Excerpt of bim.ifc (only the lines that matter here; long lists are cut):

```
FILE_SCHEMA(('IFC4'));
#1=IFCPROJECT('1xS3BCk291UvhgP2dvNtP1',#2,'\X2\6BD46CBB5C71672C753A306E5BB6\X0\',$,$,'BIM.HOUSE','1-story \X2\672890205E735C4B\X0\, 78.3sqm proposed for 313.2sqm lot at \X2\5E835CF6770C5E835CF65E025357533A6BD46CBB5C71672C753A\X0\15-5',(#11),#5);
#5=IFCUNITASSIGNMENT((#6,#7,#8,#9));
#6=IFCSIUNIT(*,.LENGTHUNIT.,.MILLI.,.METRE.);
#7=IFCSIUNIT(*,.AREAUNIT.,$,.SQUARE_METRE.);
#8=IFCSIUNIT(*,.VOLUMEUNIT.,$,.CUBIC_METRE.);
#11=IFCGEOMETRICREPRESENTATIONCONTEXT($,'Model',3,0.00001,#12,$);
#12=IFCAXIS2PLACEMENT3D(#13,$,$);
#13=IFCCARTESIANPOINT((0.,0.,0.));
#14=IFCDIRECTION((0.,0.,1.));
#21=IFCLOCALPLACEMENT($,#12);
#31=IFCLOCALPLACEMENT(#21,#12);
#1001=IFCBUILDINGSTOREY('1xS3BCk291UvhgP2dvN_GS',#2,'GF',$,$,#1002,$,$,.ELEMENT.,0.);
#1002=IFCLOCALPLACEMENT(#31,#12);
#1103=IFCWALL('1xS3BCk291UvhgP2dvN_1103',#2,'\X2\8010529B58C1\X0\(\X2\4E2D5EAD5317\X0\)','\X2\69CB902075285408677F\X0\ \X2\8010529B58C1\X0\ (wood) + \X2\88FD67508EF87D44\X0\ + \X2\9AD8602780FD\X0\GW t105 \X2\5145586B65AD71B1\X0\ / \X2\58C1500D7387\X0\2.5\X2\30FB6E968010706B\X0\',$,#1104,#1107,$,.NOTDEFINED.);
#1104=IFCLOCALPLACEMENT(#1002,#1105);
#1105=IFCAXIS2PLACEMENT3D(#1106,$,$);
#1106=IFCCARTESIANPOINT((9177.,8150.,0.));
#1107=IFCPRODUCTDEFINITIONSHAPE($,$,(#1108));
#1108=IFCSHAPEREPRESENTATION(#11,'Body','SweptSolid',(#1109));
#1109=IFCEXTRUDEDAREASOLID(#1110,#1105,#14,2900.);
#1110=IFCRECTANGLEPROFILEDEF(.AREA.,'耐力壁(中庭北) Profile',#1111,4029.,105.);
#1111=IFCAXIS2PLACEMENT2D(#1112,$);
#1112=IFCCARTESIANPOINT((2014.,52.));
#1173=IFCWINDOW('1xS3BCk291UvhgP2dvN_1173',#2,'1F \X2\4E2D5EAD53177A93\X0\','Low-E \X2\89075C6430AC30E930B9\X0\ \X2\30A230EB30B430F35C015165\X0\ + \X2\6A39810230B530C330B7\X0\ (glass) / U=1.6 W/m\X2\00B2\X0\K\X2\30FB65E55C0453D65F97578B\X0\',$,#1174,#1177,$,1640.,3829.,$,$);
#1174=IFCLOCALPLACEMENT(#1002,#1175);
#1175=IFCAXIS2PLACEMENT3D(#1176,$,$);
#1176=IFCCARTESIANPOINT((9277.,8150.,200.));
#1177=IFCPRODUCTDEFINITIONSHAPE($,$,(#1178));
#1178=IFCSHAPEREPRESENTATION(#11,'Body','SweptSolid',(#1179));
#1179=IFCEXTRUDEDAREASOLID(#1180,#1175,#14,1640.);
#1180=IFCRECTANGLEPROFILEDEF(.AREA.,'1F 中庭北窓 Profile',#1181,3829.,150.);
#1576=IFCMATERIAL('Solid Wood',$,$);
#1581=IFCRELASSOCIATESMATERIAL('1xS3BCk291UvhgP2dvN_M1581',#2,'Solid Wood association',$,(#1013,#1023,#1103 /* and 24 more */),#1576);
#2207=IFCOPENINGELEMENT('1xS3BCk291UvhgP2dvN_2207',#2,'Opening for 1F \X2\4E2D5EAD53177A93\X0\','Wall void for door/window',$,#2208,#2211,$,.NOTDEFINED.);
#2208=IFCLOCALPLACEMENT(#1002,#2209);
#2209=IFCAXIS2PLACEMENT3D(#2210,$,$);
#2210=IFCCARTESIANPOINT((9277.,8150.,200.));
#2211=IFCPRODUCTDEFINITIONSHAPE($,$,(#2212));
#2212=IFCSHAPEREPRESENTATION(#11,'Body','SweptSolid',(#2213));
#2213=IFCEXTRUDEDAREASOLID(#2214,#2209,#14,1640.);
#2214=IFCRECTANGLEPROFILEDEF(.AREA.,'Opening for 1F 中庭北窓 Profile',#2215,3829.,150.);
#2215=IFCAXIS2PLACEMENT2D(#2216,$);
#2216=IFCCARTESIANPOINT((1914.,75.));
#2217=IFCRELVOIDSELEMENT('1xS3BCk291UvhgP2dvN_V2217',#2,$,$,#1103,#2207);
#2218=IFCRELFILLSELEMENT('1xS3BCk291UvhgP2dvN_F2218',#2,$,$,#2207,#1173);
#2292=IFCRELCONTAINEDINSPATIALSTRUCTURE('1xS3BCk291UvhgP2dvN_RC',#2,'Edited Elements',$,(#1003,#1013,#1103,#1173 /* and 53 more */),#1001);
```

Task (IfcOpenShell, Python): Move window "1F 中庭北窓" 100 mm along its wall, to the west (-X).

```python
import ifcopenshell
import ifcopenshell.api.geometry
import ifcopenshell.util.placement
import ifcopenshell.util.unit

model = ifcopenshell.open("bim.ifc")
unit_scale = ifcopenshell.util.unit.calculate_unit_scale(model)

window = model.by_guid("1xS3BCk291UvhgP2dvN_1173")
opening = window.FillsVoids[0].RelatingOpeningElement
wall = opening.VoidsElements[0].RelatingBuildingElement

wall_matrix = ifcopenshell.util.placement.get_local_placement(wall.ObjectPlacement)
shift = wall_matrix[:3, 0] * -0.1 / unit_scale
before = ifcopenshell.util.placement.get_local_placement(window.ObjectPlacement)[:3, 3].copy()

# The window is not placed relative to its opening, so move both.
for product in (opening, window):
    matrix = ifcopenshell.util.placement.get_local_placement(product.ObjectPlacement)
    matrix[:3, 3] += shift
    ifcopenshell.api.geometry.edit_object_placement(model, product=product, matrix=matrix, is_si=False)

after = ifcopenshell.util.placement.get_local_placement(window.ObjectPlacement)[:3, 3]
print("window moved by", (after - before).round(3) + 0.0)

model.write("bim_v2.ifc")
```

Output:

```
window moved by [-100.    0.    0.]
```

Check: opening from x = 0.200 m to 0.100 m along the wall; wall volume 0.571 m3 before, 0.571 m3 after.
